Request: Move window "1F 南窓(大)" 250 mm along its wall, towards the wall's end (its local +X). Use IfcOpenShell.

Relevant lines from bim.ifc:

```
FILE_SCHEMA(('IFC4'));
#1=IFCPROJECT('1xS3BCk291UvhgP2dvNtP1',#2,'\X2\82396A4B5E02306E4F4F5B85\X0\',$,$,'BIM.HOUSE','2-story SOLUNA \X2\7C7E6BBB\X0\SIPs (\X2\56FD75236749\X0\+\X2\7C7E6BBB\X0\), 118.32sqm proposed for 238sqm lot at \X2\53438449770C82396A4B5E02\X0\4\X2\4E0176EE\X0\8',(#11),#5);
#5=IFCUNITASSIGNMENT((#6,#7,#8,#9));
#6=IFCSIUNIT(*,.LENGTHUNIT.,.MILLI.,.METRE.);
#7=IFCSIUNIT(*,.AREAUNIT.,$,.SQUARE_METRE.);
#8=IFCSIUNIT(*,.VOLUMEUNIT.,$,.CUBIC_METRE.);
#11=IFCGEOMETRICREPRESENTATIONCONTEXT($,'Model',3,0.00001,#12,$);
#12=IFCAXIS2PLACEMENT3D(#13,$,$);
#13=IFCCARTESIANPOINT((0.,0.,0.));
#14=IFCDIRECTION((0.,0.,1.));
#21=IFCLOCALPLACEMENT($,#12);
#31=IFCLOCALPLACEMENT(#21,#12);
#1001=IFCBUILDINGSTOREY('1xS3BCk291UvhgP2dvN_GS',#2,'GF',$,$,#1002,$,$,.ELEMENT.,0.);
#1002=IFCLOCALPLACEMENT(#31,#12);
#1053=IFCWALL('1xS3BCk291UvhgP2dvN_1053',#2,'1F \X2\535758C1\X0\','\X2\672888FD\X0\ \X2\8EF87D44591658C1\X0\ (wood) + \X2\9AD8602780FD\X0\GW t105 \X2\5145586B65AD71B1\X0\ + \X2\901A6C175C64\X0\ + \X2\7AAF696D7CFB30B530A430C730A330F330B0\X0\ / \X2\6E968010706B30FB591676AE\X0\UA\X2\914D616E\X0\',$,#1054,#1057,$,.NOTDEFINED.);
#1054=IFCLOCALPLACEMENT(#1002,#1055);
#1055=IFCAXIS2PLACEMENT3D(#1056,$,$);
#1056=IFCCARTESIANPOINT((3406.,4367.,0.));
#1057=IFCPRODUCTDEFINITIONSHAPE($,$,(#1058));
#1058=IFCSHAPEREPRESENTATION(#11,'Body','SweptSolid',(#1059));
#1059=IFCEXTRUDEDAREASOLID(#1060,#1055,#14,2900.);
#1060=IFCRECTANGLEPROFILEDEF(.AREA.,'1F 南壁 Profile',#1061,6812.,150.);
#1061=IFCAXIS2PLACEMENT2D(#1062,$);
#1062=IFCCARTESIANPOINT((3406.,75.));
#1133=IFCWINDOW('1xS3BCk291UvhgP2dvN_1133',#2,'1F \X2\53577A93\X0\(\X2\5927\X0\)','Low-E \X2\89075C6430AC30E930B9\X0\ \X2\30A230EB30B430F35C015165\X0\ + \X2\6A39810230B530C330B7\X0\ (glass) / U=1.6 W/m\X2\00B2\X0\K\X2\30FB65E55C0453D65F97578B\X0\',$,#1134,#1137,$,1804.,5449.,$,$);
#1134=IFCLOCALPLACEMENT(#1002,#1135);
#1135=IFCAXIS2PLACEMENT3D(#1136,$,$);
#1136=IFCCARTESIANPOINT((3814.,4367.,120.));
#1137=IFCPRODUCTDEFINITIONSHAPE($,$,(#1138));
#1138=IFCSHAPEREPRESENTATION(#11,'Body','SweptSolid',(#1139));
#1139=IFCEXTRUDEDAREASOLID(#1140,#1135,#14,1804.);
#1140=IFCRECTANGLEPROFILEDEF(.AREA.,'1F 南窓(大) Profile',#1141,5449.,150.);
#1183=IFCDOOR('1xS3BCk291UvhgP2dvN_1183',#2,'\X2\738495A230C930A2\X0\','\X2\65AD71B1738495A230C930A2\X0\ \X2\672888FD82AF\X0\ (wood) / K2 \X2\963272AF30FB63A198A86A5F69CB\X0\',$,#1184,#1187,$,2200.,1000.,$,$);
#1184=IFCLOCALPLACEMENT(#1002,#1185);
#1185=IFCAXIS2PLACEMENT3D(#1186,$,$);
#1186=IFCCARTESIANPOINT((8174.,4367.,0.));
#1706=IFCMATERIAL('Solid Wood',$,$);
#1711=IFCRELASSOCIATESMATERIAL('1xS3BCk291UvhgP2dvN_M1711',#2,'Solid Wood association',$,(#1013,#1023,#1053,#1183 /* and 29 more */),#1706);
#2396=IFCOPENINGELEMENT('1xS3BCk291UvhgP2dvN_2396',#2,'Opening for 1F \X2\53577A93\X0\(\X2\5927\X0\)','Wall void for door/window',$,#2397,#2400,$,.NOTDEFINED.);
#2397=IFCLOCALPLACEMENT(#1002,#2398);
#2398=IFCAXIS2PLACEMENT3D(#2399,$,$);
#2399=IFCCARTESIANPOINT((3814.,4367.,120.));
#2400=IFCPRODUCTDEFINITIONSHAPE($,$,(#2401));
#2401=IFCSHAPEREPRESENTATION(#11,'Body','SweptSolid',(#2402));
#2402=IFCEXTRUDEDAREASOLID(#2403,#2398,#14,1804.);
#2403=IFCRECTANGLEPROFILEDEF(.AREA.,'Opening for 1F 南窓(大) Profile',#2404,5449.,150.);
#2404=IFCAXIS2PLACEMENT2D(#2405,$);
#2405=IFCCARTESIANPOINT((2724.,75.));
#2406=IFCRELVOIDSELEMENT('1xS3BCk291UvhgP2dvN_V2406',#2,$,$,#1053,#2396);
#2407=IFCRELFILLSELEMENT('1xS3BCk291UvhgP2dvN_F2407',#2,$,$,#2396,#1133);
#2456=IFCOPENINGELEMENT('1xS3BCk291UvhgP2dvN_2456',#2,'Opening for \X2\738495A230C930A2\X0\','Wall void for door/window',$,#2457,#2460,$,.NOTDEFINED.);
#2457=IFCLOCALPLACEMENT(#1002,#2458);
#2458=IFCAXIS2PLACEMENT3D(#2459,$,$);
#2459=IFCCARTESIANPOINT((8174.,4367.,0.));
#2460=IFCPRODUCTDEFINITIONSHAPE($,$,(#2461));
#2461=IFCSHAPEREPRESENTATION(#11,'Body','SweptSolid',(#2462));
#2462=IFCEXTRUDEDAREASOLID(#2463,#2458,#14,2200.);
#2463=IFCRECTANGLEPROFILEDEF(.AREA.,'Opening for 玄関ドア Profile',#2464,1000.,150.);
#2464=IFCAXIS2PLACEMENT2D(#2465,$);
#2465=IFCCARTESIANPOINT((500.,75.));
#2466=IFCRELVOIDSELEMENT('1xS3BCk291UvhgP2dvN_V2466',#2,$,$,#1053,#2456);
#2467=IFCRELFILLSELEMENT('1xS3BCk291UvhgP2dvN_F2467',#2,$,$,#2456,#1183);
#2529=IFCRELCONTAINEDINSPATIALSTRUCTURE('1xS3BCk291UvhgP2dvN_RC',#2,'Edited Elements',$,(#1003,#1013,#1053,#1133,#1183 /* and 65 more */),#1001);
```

```python
import ifcopenshell
import ifcopenshell.api.geometry
import ifcopenshell.util.placement
import ifcopenshell.util.unit

model = ifcopenshell.open("bim.ifc")
unit_scale = ifcopenshell.util.unit.calculate_unit_scale(model)

window = model.by_guid("1xS3BCk291UvhgP2dvN_1133")
opening = window.FillsVoids[0].RelatingOpeningElement
wall = opening.VoidsElements[0].RelatingBuildingElement

wall_matrix = ifcopenshell.util.placement.get_local_placement(wall.ObjectPlacement)
shift = wall_matrix[:3, 0] * 0.25 / unit_scale
before = ifcopenshell.util.placement.get_local_placement(window.ObjectPlacement)[:3, 3].copy()

# The window is not placed relative to its opening, so move both.
for product in (opening, window):
    matrix = ifcopenshell.util.placement.get_local_placement(product.ObjectPlacement)
    matrix[:3, 3] += shift
    ifcopenshell.api.geometry.edit_object_placement(model, product=product, matrix=matrix, is_si=False)

after = ifcopenshell.util.placement.get_local_placement(window.ObjectPlacement)[:3, 3]
print("window moved by", (after - before).round(3) + 0.0)

model.write("bim_edited.ifc")
```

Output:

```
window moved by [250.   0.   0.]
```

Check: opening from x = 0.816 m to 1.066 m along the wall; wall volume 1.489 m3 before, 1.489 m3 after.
